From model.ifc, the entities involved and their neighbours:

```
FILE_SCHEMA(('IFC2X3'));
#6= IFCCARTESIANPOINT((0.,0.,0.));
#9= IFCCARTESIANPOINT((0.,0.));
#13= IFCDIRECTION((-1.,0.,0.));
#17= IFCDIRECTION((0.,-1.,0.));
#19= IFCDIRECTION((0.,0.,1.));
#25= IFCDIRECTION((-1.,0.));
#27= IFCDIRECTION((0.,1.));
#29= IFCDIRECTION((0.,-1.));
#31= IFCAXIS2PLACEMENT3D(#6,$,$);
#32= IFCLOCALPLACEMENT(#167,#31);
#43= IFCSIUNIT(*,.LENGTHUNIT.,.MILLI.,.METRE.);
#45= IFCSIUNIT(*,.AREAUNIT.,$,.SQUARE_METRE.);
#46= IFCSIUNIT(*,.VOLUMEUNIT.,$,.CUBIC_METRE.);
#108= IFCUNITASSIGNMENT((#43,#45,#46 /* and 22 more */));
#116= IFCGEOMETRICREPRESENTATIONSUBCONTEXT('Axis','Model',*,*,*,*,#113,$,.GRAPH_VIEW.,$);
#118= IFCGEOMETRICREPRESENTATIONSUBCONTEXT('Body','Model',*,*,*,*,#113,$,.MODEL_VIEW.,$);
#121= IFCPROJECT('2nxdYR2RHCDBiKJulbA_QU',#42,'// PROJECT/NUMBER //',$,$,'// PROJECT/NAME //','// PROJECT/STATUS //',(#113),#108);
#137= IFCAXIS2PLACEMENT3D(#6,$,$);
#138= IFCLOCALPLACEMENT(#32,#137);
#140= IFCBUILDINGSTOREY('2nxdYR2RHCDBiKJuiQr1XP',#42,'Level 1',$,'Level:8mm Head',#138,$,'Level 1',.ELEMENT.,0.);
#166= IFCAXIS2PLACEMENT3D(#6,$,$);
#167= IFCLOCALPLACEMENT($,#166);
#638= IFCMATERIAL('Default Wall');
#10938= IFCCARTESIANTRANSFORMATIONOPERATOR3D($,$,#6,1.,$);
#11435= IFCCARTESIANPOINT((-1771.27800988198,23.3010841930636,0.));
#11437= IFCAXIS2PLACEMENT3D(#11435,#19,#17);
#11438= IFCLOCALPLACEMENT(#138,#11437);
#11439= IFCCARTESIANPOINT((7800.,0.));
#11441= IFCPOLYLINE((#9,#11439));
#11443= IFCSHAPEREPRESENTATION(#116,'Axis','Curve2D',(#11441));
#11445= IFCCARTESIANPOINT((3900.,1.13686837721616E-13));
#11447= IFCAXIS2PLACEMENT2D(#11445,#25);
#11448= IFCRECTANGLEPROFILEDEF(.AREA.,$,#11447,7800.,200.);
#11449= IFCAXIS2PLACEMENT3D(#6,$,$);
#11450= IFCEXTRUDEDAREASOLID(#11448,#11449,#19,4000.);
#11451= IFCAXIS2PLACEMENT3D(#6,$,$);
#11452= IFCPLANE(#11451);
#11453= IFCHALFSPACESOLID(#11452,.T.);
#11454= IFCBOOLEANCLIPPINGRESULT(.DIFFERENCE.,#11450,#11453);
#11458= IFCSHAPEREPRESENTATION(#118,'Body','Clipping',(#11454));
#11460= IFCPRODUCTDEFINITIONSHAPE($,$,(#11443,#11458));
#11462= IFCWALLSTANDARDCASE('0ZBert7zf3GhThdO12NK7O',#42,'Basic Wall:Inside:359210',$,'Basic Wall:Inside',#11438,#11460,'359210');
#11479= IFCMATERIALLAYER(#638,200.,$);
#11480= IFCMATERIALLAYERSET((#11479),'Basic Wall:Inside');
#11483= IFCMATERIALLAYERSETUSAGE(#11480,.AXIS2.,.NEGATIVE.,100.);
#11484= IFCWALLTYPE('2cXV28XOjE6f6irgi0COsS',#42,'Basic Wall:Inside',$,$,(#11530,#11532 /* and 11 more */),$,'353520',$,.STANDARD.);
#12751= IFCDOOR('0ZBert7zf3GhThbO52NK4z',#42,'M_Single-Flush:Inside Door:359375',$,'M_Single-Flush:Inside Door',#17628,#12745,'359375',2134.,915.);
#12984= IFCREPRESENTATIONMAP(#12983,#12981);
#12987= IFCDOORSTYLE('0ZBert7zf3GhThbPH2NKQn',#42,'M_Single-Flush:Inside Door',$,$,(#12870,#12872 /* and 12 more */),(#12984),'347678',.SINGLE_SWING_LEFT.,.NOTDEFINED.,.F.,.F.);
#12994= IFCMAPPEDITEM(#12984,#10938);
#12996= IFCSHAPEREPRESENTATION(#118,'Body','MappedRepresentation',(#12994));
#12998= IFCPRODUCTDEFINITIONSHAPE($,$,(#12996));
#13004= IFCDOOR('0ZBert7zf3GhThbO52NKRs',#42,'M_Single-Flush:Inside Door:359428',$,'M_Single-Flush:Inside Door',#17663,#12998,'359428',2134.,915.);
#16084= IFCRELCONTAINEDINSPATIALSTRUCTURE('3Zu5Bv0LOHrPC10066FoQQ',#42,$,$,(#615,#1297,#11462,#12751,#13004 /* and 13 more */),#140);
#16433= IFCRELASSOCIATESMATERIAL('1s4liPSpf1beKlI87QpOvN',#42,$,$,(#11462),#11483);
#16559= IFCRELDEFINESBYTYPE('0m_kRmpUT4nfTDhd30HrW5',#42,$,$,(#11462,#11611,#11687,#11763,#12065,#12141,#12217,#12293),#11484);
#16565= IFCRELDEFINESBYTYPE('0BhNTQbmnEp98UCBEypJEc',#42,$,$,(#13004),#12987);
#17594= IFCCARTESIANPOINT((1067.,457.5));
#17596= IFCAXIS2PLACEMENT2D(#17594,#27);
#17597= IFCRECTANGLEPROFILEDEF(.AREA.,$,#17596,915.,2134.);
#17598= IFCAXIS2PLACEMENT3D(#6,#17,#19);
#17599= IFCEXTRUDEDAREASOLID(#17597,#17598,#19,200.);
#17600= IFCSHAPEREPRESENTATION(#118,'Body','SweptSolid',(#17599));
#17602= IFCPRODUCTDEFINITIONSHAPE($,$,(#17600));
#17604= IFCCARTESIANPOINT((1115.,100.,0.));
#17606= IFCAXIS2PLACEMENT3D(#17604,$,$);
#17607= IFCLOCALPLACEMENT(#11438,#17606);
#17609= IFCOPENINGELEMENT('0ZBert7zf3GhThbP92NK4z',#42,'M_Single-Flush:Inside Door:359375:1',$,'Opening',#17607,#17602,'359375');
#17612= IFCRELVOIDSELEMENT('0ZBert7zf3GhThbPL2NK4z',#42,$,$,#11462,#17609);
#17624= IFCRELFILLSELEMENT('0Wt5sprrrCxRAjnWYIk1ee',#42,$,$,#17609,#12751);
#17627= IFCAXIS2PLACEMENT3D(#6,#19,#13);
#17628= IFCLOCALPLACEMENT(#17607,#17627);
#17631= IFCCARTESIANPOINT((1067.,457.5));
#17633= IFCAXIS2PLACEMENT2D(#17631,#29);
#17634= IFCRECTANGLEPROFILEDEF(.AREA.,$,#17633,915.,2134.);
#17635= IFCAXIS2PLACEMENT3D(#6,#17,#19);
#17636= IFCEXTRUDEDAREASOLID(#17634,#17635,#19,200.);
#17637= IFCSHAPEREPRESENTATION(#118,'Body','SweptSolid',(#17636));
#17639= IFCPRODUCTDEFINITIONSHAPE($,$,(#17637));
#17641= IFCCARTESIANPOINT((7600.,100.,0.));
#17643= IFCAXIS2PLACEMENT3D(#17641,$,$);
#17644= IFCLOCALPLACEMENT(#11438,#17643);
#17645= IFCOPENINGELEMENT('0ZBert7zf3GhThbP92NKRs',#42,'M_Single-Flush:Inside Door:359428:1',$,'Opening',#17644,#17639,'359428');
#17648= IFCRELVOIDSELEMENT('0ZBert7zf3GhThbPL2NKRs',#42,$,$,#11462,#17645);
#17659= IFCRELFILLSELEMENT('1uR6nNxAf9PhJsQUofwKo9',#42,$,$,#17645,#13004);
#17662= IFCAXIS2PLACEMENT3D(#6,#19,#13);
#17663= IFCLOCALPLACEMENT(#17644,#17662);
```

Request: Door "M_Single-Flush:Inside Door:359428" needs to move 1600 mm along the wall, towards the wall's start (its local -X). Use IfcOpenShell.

```python
import ifcopenshell
import ifcopenshell.api.geometry
import ifcopenshell.util.placement
import ifcopenshell.util.unit

model = ifcopenshell.open("model.ifc")
unit_scale = ifcopenshell.util.unit.calculate_unit_scale(model)

door = model.by_guid("0ZBert7zf3GhThbO52NKRs")
opening = door.FillsVoids[0].RelatingOpeningElement
wall = opening.VoidsElements[0].RelatingBuildingElement

wall_matrix = ifcopenshell.util.placement.get_local_placement(wall.ObjectPlacement)
shift = wall_matrix[:3, 0] * -1.6 / unit_scale
before = ifcopenshell.util.placement.get_local_placement(door.ObjectPlacement)[:3, 3].copy()

# The door is placed relative to its opening, so it follows when the opening moves.
matrix = ifcopenshell.util.placement.get_local_placement(opening.ObjectPlacement)
matrix[:3, 3] += shift
ifcopenshell.api.geometry.edit_object_placement(
    model, product=opening, matrix=matrix, is_si=False, should_transform_children=True
)

after = ifcopenshell.util.placement.get_local_placement(door.ObjectPlacement)[:3, 3]
print("door moved by", (after - before).round(3) + 0.0)

model.write("model_updated.ifc")
```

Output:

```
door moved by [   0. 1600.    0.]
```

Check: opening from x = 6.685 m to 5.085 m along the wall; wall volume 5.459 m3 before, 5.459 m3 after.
